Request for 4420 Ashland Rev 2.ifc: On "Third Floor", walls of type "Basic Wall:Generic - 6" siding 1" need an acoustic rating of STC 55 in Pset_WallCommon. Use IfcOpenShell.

First a look at what the model holds.

```python
import ifcopenshell
import ifcopenshell.util.element

model = ifcopenshell.open("4420 Ashland Rev 2.ifc")
print(model.schema)
storey = next(s for s in model.by_type("IfcBuildingStorey") if s.Name == "Third Floor")
walls = [e for e in ifcopenshell.util.element.get_decomposition(storey) if e.is_a("IfcWall")]
seen = {}
for e in walls:
    element_type = ifcopenshell.util.element.get_type(e)
    key = (element_type.Name if element_type != e and element_type else None, ifcopenshell.util.element.get_pset(e, "Pset_WallCommon", "AcousticRating"))
    seen[key] = seen.get(key, 0) + 1
for (name, value), count in sorted(seen.items(), key=str):
    print(count, "x", name, "|", value)
```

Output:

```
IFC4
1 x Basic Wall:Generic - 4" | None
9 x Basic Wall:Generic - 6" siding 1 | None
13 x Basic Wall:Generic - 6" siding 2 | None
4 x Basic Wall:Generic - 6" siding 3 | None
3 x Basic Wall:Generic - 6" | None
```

```python
import ifcopenshell
import ifcopenshell.api.pset
import ifcopenshell.util.element

model = ifcopenshell.open("4420 Ashland Rev 2.ifc")

storey = next(s for s in model.by_type("IfcBuildingStorey") if s.Name == "Third Floor")
walls = [e for e in ifcopenshell.util.element.get_decomposition(storey) if e.is_a("IfcWall")]

count = 0
for e in walls:
    element_type = ifcopenshell.util.element.get_type(e)
    if element_type in (None, e) or element_type.Name != 'Basic Wall:Generic - 6" siding 1':
        continue
    # add_pset returns the element's existing set when there is one.
    pset = ifcopenshell.api.pset.add_pset(model, product=e, name="Pset_WallCommon")
    ifcopenshell.api.pset.edit_pset(model, pset=pset, properties={"AcousticRating": "STC 55"})
    count += 1

print(count, "walls updated")

model.write("4420 Ashland Rev 2_updated.ifc")
```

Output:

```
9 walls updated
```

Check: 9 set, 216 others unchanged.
